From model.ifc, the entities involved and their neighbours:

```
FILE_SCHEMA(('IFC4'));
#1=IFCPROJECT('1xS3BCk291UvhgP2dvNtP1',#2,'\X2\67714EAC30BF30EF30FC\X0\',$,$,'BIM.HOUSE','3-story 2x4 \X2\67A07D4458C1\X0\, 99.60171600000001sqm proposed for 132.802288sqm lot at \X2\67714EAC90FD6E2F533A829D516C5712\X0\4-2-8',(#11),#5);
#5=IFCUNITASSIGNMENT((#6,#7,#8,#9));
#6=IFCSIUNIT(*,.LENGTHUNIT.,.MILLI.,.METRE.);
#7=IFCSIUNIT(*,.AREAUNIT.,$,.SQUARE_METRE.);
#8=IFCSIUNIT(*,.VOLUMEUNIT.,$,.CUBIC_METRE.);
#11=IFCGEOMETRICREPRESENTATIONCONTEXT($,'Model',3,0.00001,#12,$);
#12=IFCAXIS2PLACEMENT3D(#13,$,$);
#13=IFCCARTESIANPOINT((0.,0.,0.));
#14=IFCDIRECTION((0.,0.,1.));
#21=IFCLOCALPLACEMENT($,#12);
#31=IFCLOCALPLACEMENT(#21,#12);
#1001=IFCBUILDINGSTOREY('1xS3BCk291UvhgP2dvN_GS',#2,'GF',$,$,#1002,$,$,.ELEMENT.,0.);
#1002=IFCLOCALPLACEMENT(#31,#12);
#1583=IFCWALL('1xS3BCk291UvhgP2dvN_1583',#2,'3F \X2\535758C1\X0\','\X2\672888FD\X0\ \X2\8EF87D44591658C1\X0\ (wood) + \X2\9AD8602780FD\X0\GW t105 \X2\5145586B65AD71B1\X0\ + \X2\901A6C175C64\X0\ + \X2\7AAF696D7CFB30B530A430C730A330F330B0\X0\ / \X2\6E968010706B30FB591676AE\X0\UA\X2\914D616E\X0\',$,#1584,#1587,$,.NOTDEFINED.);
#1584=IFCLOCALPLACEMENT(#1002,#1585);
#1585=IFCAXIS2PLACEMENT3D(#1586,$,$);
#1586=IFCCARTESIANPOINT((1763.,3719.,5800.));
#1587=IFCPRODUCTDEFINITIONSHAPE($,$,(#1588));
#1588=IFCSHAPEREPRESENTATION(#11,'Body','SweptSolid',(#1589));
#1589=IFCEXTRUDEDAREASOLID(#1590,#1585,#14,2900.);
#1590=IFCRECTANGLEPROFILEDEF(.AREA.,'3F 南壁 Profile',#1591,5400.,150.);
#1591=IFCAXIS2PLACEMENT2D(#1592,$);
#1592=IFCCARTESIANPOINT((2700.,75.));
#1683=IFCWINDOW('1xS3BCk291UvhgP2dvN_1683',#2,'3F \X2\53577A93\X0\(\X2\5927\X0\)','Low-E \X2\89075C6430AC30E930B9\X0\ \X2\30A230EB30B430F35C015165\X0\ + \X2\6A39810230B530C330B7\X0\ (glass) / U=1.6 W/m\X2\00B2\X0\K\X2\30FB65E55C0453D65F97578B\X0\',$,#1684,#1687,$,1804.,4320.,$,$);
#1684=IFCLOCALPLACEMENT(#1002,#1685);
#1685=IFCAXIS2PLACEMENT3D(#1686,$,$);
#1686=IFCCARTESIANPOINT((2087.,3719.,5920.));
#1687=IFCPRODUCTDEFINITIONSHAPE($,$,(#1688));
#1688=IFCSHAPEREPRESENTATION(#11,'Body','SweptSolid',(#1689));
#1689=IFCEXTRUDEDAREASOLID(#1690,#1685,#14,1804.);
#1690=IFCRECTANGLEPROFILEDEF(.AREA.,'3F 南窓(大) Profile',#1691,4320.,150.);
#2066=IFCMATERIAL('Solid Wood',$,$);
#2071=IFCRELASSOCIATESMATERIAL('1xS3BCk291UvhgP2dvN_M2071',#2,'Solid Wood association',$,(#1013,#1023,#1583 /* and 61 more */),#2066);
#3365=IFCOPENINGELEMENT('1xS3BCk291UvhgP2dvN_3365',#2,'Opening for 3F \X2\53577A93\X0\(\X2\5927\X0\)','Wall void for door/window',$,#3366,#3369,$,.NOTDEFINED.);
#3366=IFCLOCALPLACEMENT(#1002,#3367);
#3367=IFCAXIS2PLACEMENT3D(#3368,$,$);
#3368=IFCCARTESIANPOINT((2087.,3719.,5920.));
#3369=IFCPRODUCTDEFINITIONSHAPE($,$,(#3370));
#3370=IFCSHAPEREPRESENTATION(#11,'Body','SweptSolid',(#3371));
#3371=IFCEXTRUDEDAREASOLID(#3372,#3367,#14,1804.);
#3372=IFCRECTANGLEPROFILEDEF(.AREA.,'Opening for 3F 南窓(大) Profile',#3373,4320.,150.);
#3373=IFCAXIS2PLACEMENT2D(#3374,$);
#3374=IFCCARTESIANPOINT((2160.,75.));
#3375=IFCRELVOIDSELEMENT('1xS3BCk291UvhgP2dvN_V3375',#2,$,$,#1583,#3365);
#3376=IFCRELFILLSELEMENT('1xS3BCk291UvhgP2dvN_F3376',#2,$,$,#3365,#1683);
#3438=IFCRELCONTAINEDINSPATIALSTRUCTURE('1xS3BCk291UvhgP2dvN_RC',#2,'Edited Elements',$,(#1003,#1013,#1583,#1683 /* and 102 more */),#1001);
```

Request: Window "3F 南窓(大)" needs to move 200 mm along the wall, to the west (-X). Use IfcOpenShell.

```python
import ifcopenshell
import ifcopenshell.api.geometry
import ifcopenshell.util.placement
import ifcopenshell.util.unit

model = ifcopenshell.open("model.ifc")
unit_scale = ifcopenshell.util.unit.calculate_unit_scale(model)

window = model.by_guid("1xS3BCk291UvhgP2dvN_1683")
opening = window.FillsVoids[0].RelatingOpeningElement
wall = opening.VoidsElements[0].RelatingBuildingElement

wall_matrix = ifcopenshell.util.placement.get_local_placement(wall.ObjectPlacement)
shift = wall_matrix[:3, 0] * -0.2 / unit_scale
before = ifcopenshell.util.placement.get_local_placement(window.ObjectPlacement)[:3, 3].copy()

# The window is not placed relative to its opening, so move both.
for product in (opening, window):
    matrix = ifcopenshell.util.placement.get_local_placement(product.ObjectPlacement)
    matrix[:3, 3] += shift
    ifcopenshell.api.geometry.edit_object_placement(model, product=product, matrix=matrix, is_si=False)

after = ifcopenshell.util.placement.get_local_placement(window.ObjectPlacement)[:3, 3]
print("window moved by", (after - before).round(3) + 0.0)

model.write("model_v2.ifc")
```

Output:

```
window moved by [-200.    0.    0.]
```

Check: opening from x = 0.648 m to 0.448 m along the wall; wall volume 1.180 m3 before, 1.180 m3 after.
